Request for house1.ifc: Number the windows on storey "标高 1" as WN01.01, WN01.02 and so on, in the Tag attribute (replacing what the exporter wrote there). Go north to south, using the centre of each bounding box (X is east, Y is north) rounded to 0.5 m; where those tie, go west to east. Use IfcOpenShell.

First a look at what the model holds.

```python
import ifcopenshell
import ifcopenshell.util.element
import ifcopenshell.util.placement

model = ifcopenshell.open("house1.ifc")
print(model.schema)
storey = next(s for s in model.by_type("IfcBuildingStorey") if s.Name == "标高 1")
windows = [e for e in ifcopenshell.util.element.get_decomposition(storey) if e.is_a("IfcWindow")]
for e in sorted(windows, key=lambda e: e.id()):
    origin = ifcopenshell.util.placement.get_local_placement(e.ObjectPlacement)[:3, 3]
    print(e.id(), e.Tag, e.Name, origin.round(2) + 0.0, sep=" | ")
```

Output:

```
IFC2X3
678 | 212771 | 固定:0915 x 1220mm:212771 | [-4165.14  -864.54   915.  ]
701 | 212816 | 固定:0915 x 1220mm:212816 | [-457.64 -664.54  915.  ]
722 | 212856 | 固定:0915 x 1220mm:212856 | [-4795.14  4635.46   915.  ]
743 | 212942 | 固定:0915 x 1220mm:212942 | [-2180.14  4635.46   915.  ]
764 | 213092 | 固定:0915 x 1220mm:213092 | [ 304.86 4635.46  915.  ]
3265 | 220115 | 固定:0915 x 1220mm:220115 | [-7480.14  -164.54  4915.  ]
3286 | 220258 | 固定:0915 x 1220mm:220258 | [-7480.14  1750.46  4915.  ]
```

```python
import ifcopenshell
import ifcopenshell.geom
import ifcopenshell.util.element
import ifcopenshell.util.shape

model = ifcopenshell.open("house1.ifc")
settings = ifcopenshell.geom.settings()
settings.set("use-world-coords", True)


def centre(element):
    shape = ifcopenshell.geom.create_shape(settings, element)
    return ifcopenshell.util.shape.get_bbox_centroid(shape.geometry)


storey = next(s for s in model.by_type("IfcBuildingStorey") if s.Name == "标高 1")
windows = [e for e in ifcopenshell.util.element.get_decomposition(storey) if e.is_a("IfcWindow")]

# Insertion points can sit at a corner or the storey origin, so sort by the geometry (in metres).
centres = {e: centre(e) for e in windows}
windows.sort(key=lambda e: (-round(centres[e][1] / 0.5), centres[e][0]))

for i, e in enumerate(windows, start=1):
    number = f"WN01.{i:02d}"
    e.Tag = number
    print(e.id(), number)

model.write("house1_updated.ifc")
```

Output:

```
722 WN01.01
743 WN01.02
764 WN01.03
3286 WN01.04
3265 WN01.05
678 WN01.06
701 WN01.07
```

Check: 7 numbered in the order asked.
